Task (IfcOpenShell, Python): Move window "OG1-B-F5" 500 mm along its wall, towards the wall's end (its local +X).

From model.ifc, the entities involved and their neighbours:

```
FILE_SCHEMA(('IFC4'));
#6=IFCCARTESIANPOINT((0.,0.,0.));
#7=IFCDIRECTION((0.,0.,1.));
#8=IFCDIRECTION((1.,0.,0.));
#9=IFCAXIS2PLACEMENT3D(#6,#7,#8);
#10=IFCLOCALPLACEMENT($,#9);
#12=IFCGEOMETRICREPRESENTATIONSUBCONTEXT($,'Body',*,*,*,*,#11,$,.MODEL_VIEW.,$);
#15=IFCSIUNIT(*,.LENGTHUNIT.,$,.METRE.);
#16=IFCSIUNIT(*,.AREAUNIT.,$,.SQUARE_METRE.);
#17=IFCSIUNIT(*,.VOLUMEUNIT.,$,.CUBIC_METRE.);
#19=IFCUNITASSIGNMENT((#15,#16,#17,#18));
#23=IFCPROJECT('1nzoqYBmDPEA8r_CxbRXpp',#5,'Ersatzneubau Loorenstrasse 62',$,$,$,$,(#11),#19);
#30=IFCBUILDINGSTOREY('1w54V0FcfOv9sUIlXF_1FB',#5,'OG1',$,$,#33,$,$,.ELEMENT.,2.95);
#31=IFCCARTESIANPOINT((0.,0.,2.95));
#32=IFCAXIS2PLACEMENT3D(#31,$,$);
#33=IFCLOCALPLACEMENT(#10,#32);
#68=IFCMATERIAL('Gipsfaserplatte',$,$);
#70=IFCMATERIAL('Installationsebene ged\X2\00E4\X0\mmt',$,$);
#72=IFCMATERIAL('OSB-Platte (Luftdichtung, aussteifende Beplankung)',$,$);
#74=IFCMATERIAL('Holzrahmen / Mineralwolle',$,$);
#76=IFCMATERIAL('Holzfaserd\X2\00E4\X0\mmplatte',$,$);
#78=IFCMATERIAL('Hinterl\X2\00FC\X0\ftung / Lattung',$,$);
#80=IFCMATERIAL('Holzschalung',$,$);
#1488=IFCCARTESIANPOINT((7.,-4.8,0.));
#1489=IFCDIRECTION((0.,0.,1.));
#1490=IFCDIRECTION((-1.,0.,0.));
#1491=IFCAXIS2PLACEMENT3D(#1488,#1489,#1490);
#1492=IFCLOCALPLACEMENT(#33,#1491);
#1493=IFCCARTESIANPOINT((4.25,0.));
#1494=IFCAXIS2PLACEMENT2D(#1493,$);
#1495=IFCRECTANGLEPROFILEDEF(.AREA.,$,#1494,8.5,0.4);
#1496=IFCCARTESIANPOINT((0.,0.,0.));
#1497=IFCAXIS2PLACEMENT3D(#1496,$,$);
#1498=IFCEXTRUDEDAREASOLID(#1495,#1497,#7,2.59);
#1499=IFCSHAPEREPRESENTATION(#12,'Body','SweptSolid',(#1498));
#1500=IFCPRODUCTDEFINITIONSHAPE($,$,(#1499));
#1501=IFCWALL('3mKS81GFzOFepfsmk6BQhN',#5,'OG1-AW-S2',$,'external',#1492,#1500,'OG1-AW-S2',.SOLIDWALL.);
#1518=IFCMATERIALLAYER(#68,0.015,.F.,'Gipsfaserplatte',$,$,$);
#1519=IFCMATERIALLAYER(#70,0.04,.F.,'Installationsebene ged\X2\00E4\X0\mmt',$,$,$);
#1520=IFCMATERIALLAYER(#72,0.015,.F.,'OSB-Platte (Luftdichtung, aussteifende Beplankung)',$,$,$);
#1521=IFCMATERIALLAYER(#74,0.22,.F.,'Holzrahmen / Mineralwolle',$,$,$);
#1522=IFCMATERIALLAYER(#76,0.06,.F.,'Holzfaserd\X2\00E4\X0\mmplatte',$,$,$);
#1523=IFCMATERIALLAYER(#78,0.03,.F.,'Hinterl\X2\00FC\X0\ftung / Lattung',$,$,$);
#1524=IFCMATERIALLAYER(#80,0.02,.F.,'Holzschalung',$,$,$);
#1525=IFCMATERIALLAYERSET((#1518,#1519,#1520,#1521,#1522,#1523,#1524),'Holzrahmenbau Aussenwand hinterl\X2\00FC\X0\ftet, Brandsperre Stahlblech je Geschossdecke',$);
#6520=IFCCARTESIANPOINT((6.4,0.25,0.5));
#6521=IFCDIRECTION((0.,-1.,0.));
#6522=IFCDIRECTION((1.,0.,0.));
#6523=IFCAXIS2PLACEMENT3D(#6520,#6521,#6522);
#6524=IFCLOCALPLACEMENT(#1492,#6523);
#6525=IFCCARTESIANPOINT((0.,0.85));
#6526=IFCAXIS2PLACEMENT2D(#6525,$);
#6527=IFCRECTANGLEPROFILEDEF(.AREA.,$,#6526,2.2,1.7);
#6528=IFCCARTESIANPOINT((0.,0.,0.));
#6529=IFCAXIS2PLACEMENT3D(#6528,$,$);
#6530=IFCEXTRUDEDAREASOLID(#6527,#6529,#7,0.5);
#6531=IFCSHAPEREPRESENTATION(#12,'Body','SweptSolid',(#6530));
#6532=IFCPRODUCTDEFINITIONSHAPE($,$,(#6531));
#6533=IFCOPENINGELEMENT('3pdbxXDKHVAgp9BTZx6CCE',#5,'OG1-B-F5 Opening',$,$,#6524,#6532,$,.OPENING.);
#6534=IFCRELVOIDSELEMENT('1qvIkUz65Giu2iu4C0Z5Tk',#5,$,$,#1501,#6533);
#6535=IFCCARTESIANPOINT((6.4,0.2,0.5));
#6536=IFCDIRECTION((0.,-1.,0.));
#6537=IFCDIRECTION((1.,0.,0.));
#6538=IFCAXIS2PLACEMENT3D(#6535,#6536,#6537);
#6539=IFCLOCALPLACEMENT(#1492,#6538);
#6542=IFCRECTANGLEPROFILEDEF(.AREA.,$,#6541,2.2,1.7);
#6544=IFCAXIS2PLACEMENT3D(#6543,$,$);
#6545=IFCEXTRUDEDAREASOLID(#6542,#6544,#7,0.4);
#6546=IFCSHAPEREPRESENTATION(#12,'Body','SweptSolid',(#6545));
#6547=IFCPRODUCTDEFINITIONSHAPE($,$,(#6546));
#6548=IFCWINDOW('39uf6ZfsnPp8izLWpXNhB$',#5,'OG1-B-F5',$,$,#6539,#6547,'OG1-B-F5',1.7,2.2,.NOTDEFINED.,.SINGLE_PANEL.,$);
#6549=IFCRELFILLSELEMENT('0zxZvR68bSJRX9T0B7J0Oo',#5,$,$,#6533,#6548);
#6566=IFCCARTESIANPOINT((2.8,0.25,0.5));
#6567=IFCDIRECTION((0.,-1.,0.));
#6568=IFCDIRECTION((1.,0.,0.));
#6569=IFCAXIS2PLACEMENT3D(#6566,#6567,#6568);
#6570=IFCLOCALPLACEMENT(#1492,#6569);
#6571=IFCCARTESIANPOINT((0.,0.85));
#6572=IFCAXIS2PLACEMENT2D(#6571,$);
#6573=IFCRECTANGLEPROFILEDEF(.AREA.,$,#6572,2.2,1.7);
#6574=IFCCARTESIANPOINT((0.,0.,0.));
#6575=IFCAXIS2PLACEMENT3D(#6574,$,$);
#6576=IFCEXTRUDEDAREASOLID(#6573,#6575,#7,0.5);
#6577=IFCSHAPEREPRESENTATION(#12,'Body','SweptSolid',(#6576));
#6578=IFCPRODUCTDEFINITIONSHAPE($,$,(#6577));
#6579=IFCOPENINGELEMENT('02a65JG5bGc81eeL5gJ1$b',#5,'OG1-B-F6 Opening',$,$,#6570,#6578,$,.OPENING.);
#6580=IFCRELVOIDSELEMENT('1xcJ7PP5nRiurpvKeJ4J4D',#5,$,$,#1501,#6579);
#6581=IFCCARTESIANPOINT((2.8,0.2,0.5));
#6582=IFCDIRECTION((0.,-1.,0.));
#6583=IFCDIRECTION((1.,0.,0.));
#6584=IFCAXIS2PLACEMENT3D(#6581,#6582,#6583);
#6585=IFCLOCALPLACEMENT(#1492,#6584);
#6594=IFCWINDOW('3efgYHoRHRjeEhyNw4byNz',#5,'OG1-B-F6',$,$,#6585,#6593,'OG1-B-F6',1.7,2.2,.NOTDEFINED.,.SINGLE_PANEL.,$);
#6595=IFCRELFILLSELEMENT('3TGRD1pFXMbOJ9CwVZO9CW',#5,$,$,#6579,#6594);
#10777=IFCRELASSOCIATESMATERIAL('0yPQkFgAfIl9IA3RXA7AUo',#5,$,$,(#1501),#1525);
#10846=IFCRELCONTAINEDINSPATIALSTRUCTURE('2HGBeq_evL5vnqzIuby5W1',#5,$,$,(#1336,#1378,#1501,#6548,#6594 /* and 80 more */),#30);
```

```python
import ifcopenshell
import ifcopenshell.api.geometry
import ifcopenshell.util.placement
import ifcopenshell.util.unit

model = ifcopenshell.open("model.ifc")
unit_scale = ifcopenshell.util.unit.calculate_unit_scale(model)

window = model.by_guid("39uf6ZfsnPp8izLWpXNhB$")
opening = window.FillsVoids[0].RelatingOpeningElement
wall = opening.VoidsElements[0].RelatingBuildingElement

wall_matrix = ifcopenshell.util.placement.get_local_placement(wall.ObjectPlacement)
shift = wall_matrix[:3, 0] * 0.5 / unit_scale
before = ifcopenshell.util.placement.get_local_placement(window.ObjectPlacement)[:3, 3].copy()

# The window is not placed relative to its opening, so move both.
for product in (opening, window):
    matrix = ifcopenshell.util.placement.get_local_placement(product.ObjectPlacement)
    matrix[:3, 3] += shift
    ifcopenshell.api.geometry.edit_object_placement(model, product=product, matrix=matrix, is_si=False)

after = ifcopenshell.util.placement.get_local_placement(window.ObjectPlacement)[:3, 3]
print("window moved by", (after - before).round(3) + 0.0)

model.write("model_edited.ifc")
```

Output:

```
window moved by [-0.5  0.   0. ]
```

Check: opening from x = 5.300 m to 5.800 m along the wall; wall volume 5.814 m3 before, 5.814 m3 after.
